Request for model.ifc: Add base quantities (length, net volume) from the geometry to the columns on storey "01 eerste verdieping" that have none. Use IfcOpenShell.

First a look at what the model holds.

```python
import ifcopenshell
import ifcopenshell.util.element
import ifcopenshell.util.unit

model = ifcopenshell.open("model.ifc")
print(model.schema)
for unit_type in ("LENGTHUNIT", "AREAUNIT", "VOLUMEUNIT"):
    print(unit_type, ifcopenshell.util.unit.calculate_unit_scale(model, unit_type))
storey = next(s for s in model.by_type("IfcBuildingStorey") if s.Name == "01 eerste verdieping")
columns = [e for e in ifcopenshell.util.element.get_decomposition(storey) if e.is_a("IfcColumn")]
for e in sorted(columns, key=lambda e: e.id()):
    print(e.id(), e.is_a(), e.Name, list(ifcopenshell.util.element.get_psets(e, qtos_only=True)), sep=" | ")
```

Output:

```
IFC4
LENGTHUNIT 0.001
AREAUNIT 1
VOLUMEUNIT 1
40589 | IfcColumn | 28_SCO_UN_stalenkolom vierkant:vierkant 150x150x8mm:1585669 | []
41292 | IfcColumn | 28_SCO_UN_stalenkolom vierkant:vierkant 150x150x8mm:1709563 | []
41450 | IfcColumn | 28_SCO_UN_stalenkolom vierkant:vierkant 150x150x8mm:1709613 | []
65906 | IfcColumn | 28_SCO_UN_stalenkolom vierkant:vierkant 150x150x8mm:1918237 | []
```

```python
import ifcopenshell
import ifcopenshell.api.pset
import ifcopenshell.geom
import ifcopenshell.util.element
import ifcopenshell.util.shape
import ifcopenshell.util.unit

model = ifcopenshell.open("model.ifc")
unit_scale = ifcopenshell.util.unit.calculate_unit_scale(model)
volume_scale = ifcopenshell.util.unit.calculate_unit_scale(model, "VOLUMEUNIT")
settings = ifcopenshell.geom.settings()

storey = next(s for s in model.by_type("IfcBuildingStorey") if s.Name == "01 eerste verdieping")
columns = [e for e in ifcopenshell.util.element.get_decomposition(storey) if e.is_a("IfcColumn")]

for e in sorted(columns, key=lambda e: e.id()):
    if ifcopenshell.util.element.get_psets(e, qtos_only=True, should_inherit=False):
        continue
    # Geometry comes back in metres, in the element's own axes.
    shape = ifcopenshell.geom.create_shape(settings, e)
    values = {
        "Length": ifcopenshell.util.shape.get_z(shape.geometry) / unit_scale,
        "NetVolume": ifcopenshell.util.shape.get_volume(shape.geometry) / volume_scale,
    }
    qto = ifcopenshell.api.pset.add_qto(model, product=e, name="Qto_ColumnBaseQuantities")
    ifcopenshell.api.pset.edit_qto(model, qto=qto, properties=values)
    print(e.id(), {k: round(v, 3) for k, v in values.items()})

model.write("model_rev.ifc")
```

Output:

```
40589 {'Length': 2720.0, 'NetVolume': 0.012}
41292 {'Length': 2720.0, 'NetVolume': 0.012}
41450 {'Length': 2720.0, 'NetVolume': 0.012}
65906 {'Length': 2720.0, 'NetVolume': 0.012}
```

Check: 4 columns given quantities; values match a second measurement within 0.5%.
